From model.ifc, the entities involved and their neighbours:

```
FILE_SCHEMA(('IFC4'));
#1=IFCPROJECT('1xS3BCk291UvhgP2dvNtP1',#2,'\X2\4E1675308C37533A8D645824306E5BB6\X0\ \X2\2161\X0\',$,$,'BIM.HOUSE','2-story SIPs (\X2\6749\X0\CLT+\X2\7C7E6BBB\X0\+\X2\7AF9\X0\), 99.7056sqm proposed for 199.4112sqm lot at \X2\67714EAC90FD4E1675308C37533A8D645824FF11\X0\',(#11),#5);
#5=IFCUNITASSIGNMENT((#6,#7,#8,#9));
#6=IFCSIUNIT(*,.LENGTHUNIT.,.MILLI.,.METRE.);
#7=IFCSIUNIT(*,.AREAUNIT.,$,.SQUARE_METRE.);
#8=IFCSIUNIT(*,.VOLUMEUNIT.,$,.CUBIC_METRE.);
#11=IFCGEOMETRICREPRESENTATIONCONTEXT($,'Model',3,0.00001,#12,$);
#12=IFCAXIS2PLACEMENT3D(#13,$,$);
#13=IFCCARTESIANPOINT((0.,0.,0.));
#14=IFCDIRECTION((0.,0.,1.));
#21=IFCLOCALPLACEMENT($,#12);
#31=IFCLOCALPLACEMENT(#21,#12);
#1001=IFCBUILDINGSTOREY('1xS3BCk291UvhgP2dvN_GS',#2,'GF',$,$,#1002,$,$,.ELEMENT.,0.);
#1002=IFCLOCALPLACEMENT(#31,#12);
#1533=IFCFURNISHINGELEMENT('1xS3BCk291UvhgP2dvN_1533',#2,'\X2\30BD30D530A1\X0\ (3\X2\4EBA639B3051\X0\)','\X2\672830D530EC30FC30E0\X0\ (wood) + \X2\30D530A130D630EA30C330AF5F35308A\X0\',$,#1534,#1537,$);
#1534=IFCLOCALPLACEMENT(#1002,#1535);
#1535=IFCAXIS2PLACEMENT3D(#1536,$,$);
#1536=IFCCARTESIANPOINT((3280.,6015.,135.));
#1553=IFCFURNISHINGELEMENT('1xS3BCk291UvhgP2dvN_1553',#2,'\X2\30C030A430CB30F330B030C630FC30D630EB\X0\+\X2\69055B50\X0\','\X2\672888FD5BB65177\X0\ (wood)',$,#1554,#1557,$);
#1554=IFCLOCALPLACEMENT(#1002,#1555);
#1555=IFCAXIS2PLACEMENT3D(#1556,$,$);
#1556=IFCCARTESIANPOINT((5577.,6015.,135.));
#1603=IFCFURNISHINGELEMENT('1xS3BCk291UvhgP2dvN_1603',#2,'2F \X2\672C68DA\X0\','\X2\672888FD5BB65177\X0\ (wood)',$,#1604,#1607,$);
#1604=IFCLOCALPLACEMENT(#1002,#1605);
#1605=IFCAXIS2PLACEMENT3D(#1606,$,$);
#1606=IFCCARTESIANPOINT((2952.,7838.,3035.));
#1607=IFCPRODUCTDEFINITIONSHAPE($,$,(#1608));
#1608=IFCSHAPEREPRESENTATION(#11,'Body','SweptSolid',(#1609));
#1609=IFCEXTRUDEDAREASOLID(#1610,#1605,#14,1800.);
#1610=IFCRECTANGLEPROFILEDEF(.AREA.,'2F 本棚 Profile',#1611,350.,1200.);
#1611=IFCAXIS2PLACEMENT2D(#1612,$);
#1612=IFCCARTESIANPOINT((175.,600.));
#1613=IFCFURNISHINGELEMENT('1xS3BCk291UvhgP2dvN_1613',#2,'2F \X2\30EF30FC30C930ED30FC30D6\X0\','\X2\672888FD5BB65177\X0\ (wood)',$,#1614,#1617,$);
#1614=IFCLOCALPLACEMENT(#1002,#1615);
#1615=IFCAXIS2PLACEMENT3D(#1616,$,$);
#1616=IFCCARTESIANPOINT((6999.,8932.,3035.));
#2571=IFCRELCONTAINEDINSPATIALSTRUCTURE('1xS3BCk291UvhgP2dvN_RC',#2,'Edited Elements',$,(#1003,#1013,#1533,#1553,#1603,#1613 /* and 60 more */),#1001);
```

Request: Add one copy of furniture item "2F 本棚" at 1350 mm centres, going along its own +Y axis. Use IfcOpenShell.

```python
import ifcopenshell
import ifcopenshell.api.geometry
import ifcopenshell.api.root
import ifcopenshell.util.element
import ifcopenshell.util.placement

model = ifcopenshell.open("model.ifc")


def reuse_history(source, copy):
    """copy_class also copies each property set's owner history, people and application; keep the originals."""
    for rel in copy.IsDefinedBy:
        if rel.is_a("IfcRelDefinesByProperties") and (history := rel.RelatingPropertyDefinition.OwnerHistory):
            rel.RelatingPropertyDefinition.OwnerHistory = source.OwnerHistory
            ifcopenshell.util.element.remove_deep2(model, history)


source = model.by_guid("1xS3BCk291UvhgP2dvN_1603")
base = ifcopenshell.util.placement.get_local_placement(source.ObjectPlacement)
step = base[:3, 1] * 1350.0

for i in range(1, 2):
    copy = ifcopenshell.api.root.copy_class(model, product=source)
    copy.Representation = ifcopenshell.util.element.copy_deep(
        model, source.Representation, exclude=["IfcGeometricRepresentationContext", "IfcRepresentationMap"]
    )
    reuse_history(source, copy)
    matrix = base.copy()
    matrix[:3, 3] += i * step
    print("added at", matrix[:3, 3].round(3) + 0.0)
    ifcopenshell.api.geometry.edit_object_placement(model, product=copy, matrix=matrix, is_si=False)

model.write("model_updated.ifc")
```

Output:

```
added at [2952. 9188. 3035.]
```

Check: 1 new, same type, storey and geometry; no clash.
